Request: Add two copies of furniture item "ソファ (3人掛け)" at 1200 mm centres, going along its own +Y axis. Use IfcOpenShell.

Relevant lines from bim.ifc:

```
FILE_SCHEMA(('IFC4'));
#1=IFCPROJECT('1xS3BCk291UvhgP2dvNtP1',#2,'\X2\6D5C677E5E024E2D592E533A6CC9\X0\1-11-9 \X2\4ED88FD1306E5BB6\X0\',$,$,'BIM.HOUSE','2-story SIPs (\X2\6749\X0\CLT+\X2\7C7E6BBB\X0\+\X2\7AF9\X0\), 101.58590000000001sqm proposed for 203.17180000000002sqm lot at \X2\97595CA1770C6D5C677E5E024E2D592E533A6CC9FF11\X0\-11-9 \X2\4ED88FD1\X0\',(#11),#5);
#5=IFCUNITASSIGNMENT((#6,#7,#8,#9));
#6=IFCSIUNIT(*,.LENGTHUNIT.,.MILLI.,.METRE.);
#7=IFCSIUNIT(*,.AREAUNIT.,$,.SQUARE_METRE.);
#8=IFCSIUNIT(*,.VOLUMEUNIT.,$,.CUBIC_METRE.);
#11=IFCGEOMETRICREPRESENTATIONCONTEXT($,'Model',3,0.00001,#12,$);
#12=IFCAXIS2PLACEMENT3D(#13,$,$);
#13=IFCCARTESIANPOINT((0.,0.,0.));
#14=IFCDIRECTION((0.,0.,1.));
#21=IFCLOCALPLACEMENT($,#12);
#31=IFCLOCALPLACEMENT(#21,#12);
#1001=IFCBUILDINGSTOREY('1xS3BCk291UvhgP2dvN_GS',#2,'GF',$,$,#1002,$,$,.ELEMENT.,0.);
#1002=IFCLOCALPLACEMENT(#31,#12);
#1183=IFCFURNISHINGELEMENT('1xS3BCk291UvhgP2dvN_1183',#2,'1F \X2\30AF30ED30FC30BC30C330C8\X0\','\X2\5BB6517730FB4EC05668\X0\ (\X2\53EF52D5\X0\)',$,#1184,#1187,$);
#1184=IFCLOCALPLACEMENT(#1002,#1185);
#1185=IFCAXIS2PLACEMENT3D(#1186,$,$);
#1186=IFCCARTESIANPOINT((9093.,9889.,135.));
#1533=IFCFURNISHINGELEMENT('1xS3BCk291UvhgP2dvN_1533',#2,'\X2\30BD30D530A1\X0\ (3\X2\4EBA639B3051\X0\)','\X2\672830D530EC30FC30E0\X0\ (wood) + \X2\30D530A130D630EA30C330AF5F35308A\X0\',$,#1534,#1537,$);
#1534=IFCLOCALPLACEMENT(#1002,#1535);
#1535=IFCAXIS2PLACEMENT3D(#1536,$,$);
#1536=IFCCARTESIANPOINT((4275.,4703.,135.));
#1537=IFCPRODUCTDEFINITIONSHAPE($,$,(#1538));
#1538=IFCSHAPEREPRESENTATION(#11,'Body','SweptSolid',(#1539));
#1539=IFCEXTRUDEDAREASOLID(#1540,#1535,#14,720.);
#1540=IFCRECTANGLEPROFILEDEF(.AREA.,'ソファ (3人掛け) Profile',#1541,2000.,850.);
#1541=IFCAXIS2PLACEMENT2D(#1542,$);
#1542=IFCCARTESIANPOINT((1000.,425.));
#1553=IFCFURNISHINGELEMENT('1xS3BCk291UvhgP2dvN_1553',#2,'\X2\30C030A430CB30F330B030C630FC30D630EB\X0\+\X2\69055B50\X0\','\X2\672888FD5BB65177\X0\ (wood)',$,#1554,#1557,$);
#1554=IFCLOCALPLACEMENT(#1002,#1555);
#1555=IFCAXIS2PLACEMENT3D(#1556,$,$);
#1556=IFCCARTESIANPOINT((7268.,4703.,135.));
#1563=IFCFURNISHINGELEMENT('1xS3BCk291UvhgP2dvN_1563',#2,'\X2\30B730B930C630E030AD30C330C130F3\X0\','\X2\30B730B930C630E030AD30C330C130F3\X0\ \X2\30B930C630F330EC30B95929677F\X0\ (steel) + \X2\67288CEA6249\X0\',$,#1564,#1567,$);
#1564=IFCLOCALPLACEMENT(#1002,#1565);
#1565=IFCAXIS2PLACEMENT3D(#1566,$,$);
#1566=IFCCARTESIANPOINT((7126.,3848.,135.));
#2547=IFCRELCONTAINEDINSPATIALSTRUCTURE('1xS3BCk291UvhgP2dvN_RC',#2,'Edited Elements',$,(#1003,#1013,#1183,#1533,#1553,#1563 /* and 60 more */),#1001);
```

```python
import ifcopenshell
import ifcopenshell.api.geometry
import ifcopenshell.api.root
import ifcopenshell.util.element
import ifcopenshell.util.placement
import ifcopenshell.util.unit

model = ifcopenshell.open("bim.ifc")
unit_scale = ifcopenshell.util.unit.calculate_unit_scale(model)


def reuse_history(source, copy):
    """copy_class also copies each property set's owner history, people and application; keep the originals."""
    for rel in copy.IsDefinedBy:
        if rel.is_a("IfcRelDefinesByProperties") and (history := rel.RelatingPropertyDefinition.OwnerHistory):
            rel.RelatingPropertyDefinition.OwnerHistory = source.OwnerHistory
            ifcopenshell.util.element.remove_deep2(model, history)


source = model.by_guid("1xS3BCk291UvhgP2dvN_1533")
base = ifcopenshell.util.placement.get_local_placement(source.ObjectPlacement)
step = base[:3, 1] * 1.2 / unit_scale

for i in range(1, 3):
    copy = ifcopenshell.api.root.copy_class(model, product=source)
    copy.Representation = ifcopenshell.util.element.copy_deep(
        model, source.Representation, exclude=["IfcGeometricRepresentationContext", "IfcRepresentationMap"]
    )
    reuse_history(source, copy)
    matrix = base.copy()
    matrix[:3, 3] += i * step
    print("added at", matrix[:3, 3].round(3) + 0.0)
    ifcopenshell.api.geometry.edit_object_placement(model, product=copy, matrix=matrix, is_si=False)

model.write("bim_v2.ifc")
```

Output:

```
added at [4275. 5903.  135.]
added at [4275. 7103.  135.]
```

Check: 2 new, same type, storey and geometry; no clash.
